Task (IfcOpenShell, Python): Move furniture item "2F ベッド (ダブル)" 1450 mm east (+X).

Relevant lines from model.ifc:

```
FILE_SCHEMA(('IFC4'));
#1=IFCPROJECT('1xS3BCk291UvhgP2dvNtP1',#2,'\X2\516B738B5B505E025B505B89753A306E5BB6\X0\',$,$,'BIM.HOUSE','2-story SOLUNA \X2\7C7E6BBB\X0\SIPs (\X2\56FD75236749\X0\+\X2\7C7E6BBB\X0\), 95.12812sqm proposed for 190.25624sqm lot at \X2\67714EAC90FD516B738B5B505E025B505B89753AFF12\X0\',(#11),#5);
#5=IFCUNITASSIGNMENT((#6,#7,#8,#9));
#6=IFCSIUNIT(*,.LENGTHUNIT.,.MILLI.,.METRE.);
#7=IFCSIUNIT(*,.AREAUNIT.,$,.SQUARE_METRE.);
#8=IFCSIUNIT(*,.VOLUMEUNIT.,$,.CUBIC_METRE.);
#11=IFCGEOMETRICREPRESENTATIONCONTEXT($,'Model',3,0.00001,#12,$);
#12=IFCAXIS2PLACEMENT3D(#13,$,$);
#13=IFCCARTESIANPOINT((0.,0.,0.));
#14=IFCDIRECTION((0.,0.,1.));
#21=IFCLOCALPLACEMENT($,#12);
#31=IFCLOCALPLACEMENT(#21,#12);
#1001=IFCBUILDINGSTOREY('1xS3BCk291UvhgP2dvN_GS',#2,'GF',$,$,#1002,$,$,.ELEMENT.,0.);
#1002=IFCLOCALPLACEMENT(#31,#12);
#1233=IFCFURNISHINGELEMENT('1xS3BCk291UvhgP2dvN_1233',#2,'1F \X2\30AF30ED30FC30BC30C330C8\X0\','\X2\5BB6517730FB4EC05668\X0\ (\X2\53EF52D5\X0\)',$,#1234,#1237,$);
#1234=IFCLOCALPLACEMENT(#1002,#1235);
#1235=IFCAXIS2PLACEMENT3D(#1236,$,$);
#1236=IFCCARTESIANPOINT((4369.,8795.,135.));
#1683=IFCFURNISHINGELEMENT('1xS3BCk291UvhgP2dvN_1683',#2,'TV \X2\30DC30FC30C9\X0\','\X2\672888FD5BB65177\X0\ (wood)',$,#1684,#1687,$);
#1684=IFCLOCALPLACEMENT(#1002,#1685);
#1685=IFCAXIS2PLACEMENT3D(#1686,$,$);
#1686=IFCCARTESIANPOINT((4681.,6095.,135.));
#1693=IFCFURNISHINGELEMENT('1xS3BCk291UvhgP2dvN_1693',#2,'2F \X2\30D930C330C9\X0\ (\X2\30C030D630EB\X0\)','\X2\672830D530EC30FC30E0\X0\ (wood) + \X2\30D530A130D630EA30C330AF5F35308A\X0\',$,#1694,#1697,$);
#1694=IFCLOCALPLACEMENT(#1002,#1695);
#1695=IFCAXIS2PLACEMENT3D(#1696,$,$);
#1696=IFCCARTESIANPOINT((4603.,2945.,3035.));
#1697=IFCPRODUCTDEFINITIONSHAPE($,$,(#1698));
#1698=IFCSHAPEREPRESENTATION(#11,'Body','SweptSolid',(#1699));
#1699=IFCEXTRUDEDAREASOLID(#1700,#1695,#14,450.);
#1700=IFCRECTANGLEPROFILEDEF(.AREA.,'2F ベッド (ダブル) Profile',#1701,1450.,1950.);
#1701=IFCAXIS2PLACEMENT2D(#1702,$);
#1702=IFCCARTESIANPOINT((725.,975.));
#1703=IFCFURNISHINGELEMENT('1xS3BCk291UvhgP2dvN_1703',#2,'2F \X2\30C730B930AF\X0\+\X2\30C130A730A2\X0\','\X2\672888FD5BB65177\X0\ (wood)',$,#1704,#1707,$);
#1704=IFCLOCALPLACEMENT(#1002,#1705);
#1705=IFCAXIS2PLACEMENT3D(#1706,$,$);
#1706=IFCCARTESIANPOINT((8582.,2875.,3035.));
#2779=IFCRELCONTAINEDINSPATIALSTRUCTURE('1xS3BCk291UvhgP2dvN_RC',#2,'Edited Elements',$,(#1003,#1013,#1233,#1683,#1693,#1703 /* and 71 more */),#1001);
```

```python
import ifcopenshell
import ifcopenshell.api.geometry
import ifcopenshell.util.placement
import ifcopenshell.util.unit

model = ifcopenshell.open("model.ifc")
unit_scale = ifcopenshell.util.unit.calculate_unit_scale(model)

item = model.by_guid("1xS3BCk291UvhgP2dvN_1693")
matrix = ifcopenshell.util.placement.get_local_placement(item.ObjectPlacement)
matrix[0, 3] += 1.45 / unit_scale
ifcopenshell.api.geometry.edit_object_placement(model, product=item, matrix=matrix, is_si=False)

print(ifcopenshell.util.placement.get_local_placement(item.ObjectPlacement).round(3) + 0.0)

model.write("model_updated.ifc")
```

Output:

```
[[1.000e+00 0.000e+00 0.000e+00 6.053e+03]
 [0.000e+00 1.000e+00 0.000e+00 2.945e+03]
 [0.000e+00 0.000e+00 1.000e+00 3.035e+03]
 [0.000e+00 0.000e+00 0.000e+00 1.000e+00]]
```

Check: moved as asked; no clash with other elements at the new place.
